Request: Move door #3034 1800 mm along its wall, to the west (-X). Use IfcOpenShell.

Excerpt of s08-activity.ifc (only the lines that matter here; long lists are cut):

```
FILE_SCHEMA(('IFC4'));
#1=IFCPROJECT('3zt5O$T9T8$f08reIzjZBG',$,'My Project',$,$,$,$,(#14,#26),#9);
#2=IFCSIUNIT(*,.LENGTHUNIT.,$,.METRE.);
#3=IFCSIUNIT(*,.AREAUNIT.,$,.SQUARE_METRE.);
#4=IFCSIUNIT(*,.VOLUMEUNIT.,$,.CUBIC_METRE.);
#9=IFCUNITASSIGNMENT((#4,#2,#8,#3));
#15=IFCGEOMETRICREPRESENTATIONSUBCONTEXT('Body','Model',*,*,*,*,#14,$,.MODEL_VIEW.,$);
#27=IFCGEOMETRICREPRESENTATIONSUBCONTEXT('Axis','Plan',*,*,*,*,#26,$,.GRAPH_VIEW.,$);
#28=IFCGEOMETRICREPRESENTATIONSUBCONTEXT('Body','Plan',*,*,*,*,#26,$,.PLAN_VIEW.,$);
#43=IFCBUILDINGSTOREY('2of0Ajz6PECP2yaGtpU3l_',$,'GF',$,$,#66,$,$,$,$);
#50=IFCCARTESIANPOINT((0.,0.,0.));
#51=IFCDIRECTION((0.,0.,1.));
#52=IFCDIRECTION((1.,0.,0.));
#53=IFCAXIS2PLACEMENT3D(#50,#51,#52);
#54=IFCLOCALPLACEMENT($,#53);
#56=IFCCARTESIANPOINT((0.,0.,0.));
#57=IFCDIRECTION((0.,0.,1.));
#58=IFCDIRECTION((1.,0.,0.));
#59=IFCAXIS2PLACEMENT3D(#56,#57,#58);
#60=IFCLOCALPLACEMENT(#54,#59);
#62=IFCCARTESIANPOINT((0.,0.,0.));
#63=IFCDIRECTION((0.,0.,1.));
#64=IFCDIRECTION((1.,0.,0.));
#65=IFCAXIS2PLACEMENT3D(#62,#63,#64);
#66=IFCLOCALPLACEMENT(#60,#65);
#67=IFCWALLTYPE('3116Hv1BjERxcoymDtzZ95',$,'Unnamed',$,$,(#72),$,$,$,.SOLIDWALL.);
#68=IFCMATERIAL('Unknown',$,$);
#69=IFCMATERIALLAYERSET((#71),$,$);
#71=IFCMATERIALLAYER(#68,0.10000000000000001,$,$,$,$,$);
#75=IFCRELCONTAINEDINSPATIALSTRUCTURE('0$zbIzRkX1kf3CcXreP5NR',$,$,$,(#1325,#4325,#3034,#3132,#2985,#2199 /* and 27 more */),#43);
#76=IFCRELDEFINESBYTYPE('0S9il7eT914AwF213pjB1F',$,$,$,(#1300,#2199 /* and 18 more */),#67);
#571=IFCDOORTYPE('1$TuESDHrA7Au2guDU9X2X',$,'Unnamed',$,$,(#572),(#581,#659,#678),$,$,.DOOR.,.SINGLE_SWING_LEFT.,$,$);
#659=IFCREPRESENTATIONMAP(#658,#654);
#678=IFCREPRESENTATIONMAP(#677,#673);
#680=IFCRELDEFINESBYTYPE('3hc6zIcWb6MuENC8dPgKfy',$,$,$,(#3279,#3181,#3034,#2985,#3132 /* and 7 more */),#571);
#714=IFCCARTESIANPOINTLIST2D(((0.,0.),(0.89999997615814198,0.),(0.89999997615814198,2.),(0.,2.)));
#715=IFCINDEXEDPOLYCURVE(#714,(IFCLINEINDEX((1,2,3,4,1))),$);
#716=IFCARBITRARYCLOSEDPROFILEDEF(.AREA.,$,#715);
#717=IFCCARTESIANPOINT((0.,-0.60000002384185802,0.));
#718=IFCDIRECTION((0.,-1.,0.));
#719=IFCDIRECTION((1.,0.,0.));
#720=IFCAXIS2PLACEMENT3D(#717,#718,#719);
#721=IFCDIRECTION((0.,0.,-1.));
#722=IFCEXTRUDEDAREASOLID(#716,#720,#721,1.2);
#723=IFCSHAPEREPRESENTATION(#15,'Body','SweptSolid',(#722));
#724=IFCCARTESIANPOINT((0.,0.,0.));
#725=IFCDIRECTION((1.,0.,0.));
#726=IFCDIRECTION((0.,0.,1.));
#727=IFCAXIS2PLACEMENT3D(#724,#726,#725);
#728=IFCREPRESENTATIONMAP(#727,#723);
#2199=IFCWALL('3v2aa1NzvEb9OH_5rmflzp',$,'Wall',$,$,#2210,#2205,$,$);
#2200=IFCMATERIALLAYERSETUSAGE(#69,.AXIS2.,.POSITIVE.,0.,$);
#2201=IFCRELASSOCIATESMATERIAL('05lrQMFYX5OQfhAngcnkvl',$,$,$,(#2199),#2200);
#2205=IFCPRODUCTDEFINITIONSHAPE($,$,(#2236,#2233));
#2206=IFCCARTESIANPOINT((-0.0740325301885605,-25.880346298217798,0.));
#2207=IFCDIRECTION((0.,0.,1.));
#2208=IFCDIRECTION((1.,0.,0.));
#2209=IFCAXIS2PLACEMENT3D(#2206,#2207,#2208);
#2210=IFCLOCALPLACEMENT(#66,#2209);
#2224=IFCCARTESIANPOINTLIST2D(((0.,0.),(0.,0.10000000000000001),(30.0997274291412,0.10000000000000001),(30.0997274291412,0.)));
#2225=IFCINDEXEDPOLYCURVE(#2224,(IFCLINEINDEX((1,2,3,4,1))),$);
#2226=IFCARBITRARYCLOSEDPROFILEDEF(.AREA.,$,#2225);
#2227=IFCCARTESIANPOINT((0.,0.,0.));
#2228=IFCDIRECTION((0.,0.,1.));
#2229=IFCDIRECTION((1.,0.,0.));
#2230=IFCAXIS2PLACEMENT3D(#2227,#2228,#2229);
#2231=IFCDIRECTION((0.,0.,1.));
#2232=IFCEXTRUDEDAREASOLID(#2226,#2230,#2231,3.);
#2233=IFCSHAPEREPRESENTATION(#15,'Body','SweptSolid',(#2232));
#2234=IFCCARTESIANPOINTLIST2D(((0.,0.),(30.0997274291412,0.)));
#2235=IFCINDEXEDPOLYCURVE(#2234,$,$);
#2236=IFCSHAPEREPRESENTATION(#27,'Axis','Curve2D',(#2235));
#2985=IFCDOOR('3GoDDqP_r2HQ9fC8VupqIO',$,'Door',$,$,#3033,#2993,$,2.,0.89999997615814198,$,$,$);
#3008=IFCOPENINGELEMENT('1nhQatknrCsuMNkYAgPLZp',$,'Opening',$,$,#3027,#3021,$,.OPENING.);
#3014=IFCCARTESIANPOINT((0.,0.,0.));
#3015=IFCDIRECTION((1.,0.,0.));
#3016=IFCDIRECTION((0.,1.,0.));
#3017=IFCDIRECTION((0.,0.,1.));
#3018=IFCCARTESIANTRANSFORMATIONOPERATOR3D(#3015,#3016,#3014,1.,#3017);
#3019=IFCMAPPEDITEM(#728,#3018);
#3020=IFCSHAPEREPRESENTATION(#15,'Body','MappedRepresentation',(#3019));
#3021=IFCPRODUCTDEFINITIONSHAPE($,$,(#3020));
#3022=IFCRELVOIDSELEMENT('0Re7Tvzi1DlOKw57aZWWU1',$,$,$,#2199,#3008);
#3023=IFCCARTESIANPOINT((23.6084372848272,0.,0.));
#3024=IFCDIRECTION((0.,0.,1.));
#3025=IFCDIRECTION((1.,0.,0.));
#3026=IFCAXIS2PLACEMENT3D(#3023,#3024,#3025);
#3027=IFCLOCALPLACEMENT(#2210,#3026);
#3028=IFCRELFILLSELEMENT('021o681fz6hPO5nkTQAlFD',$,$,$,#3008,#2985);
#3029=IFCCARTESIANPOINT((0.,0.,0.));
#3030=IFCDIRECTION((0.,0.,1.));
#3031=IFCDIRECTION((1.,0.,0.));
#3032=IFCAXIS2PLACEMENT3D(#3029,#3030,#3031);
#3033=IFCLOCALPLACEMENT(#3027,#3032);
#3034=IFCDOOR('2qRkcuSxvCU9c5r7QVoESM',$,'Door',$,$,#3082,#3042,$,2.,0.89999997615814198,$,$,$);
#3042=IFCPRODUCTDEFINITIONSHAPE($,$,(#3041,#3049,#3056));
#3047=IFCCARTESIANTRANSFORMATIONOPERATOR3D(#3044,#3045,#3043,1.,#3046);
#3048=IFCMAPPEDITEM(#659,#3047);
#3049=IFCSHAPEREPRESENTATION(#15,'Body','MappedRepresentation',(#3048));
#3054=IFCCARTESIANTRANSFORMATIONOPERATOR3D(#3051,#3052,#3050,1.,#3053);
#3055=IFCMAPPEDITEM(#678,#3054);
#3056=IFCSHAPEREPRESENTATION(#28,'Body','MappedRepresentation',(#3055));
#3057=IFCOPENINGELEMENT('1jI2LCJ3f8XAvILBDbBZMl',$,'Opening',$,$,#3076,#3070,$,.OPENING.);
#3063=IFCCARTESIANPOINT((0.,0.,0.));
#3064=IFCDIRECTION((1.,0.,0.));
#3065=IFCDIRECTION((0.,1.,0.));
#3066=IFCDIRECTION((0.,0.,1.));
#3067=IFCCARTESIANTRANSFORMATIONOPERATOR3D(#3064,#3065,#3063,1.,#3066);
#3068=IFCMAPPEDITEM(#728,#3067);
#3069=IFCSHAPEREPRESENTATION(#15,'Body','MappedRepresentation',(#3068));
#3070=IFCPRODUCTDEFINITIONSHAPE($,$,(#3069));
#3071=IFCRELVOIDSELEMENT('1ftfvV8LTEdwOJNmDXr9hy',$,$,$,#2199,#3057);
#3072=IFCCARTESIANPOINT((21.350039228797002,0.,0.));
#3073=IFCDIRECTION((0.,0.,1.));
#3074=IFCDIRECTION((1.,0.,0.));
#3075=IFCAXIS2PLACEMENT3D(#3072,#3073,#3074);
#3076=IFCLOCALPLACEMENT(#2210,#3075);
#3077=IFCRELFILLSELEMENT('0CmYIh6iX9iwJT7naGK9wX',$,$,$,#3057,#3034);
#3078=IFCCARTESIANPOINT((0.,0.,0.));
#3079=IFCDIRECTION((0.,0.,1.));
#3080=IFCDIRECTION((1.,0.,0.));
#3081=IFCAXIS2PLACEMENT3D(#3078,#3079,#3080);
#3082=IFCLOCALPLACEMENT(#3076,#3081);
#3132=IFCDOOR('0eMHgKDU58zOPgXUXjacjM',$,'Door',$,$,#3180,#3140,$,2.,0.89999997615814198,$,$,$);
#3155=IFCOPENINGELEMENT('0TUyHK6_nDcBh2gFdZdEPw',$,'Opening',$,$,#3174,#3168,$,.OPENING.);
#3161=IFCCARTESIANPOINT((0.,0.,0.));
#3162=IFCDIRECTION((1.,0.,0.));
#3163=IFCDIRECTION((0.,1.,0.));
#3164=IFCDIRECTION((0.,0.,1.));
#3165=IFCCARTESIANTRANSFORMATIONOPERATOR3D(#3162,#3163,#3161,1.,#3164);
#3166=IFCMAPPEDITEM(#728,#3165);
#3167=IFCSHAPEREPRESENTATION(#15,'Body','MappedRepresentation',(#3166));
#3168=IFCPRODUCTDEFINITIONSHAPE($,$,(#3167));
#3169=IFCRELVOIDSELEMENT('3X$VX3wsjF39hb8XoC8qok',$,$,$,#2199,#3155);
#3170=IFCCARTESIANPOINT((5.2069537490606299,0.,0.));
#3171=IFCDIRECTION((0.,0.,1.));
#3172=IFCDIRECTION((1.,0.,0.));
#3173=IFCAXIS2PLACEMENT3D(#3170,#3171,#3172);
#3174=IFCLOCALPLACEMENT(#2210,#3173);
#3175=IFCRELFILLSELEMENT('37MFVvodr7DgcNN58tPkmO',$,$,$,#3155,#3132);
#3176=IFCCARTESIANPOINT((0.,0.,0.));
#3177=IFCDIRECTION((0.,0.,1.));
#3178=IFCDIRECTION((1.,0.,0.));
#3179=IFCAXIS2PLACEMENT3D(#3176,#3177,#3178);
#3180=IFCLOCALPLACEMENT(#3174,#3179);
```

```python
import ifcopenshell
import ifcopenshell.api.geometry
import ifcopenshell.util.placement

model = ifcopenshell.open("s08-activity.ifc")

door = model.by_id(3034)
opening = door.FillsVoids[0].RelatingOpeningElement
wall = opening.VoidsElements[0].RelatingBuildingElement

wall_matrix = ifcopenshell.util.placement.get_local_placement(wall.ObjectPlacement)
shift = wall_matrix[:3, 0] * -1.8
before = ifcopenshell.util.placement.get_local_placement(door.ObjectPlacement)[:3, 3].copy()

# The door is placed relative to its opening, so it follows when the opening moves.
matrix = ifcopenshell.util.placement.get_local_placement(opening.ObjectPlacement)
matrix[:3, 3] += shift
ifcopenshell.api.geometry.edit_object_placement(
    model, product=opening, matrix=matrix, is_si=False, should_transform_children=True
)

after = ifcopenshell.util.placement.get_local_placement(door.ObjectPlacement)[:3, 3]
print("door moved by", (after - before).round(3) + 0.0)

model.write("s08-activity-out.ifc")
```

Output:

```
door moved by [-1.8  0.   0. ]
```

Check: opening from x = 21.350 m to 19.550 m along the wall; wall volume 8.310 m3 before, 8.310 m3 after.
